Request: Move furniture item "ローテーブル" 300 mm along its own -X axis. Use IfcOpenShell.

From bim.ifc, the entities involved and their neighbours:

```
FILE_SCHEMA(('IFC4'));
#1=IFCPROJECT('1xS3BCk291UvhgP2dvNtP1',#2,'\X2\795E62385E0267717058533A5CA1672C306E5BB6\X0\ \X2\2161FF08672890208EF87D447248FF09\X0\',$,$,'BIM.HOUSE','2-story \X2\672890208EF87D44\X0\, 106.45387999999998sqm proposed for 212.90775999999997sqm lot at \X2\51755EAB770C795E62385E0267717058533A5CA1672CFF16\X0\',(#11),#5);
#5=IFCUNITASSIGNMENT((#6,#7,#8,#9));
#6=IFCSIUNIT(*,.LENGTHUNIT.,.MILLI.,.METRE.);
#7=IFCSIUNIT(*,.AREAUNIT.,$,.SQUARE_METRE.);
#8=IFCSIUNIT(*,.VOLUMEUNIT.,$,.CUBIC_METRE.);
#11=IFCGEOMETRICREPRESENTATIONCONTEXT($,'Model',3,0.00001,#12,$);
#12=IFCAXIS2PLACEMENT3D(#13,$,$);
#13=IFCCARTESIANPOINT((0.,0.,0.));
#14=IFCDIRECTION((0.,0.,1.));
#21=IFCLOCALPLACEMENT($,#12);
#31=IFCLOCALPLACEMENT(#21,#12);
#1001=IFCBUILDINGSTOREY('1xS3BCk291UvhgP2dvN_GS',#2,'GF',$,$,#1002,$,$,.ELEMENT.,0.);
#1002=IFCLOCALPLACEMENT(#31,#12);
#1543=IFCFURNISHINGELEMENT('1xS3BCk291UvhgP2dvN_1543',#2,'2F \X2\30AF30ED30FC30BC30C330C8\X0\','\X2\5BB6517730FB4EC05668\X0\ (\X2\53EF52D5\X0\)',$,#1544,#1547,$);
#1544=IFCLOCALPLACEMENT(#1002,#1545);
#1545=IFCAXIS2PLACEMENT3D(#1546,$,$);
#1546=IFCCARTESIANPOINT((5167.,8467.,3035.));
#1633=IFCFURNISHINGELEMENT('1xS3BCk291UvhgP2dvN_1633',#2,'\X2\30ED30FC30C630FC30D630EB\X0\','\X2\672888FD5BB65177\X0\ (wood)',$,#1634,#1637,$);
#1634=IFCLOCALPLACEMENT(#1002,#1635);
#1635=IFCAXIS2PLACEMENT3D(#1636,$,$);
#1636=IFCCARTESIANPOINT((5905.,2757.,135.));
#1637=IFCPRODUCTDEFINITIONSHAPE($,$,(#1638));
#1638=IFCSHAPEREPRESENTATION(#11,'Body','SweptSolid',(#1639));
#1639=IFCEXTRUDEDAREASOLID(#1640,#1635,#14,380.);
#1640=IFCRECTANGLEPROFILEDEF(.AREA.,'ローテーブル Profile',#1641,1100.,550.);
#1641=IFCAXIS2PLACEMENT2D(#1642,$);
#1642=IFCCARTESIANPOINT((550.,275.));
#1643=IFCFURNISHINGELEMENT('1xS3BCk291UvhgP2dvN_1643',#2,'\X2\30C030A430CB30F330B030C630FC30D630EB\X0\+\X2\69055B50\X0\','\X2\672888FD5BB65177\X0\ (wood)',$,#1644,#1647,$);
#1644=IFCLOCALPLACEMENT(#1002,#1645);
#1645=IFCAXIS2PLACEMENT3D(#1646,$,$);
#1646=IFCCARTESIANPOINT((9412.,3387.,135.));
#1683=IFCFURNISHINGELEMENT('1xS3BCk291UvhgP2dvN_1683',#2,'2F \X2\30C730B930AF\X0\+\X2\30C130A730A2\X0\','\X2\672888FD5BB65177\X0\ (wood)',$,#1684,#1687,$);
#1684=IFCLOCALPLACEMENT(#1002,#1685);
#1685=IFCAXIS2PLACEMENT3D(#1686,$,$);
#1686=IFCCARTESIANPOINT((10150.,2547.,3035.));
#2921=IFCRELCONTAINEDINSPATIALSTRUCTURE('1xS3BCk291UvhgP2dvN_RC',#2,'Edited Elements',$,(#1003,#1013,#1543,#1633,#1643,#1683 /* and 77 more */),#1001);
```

```python
import ifcopenshell
import ifcopenshell.api.geometry
import ifcopenshell.util.placement

model = ifcopenshell.open("bim.ifc")

item = model.by_guid("1xS3BCk291UvhgP2dvN_1633")
matrix = ifcopenshell.util.placement.get_local_placement(item.ObjectPlacement)
matrix[:3, 3] -= matrix[:3, 0] * 300.0
ifcopenshell.api.geometry.edit_object_placement(model, product=item, matrix=matrix, is_si=False)

print(ifcopenshell.util.placement.get_local_placement(item.ObjectPlacement).round(3) + 0.0)

model.write("bim_edited.ifc")
```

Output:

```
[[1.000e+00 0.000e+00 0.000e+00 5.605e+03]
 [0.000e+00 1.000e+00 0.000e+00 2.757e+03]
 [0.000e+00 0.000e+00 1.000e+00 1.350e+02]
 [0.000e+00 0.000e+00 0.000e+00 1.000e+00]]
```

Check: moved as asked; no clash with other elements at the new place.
